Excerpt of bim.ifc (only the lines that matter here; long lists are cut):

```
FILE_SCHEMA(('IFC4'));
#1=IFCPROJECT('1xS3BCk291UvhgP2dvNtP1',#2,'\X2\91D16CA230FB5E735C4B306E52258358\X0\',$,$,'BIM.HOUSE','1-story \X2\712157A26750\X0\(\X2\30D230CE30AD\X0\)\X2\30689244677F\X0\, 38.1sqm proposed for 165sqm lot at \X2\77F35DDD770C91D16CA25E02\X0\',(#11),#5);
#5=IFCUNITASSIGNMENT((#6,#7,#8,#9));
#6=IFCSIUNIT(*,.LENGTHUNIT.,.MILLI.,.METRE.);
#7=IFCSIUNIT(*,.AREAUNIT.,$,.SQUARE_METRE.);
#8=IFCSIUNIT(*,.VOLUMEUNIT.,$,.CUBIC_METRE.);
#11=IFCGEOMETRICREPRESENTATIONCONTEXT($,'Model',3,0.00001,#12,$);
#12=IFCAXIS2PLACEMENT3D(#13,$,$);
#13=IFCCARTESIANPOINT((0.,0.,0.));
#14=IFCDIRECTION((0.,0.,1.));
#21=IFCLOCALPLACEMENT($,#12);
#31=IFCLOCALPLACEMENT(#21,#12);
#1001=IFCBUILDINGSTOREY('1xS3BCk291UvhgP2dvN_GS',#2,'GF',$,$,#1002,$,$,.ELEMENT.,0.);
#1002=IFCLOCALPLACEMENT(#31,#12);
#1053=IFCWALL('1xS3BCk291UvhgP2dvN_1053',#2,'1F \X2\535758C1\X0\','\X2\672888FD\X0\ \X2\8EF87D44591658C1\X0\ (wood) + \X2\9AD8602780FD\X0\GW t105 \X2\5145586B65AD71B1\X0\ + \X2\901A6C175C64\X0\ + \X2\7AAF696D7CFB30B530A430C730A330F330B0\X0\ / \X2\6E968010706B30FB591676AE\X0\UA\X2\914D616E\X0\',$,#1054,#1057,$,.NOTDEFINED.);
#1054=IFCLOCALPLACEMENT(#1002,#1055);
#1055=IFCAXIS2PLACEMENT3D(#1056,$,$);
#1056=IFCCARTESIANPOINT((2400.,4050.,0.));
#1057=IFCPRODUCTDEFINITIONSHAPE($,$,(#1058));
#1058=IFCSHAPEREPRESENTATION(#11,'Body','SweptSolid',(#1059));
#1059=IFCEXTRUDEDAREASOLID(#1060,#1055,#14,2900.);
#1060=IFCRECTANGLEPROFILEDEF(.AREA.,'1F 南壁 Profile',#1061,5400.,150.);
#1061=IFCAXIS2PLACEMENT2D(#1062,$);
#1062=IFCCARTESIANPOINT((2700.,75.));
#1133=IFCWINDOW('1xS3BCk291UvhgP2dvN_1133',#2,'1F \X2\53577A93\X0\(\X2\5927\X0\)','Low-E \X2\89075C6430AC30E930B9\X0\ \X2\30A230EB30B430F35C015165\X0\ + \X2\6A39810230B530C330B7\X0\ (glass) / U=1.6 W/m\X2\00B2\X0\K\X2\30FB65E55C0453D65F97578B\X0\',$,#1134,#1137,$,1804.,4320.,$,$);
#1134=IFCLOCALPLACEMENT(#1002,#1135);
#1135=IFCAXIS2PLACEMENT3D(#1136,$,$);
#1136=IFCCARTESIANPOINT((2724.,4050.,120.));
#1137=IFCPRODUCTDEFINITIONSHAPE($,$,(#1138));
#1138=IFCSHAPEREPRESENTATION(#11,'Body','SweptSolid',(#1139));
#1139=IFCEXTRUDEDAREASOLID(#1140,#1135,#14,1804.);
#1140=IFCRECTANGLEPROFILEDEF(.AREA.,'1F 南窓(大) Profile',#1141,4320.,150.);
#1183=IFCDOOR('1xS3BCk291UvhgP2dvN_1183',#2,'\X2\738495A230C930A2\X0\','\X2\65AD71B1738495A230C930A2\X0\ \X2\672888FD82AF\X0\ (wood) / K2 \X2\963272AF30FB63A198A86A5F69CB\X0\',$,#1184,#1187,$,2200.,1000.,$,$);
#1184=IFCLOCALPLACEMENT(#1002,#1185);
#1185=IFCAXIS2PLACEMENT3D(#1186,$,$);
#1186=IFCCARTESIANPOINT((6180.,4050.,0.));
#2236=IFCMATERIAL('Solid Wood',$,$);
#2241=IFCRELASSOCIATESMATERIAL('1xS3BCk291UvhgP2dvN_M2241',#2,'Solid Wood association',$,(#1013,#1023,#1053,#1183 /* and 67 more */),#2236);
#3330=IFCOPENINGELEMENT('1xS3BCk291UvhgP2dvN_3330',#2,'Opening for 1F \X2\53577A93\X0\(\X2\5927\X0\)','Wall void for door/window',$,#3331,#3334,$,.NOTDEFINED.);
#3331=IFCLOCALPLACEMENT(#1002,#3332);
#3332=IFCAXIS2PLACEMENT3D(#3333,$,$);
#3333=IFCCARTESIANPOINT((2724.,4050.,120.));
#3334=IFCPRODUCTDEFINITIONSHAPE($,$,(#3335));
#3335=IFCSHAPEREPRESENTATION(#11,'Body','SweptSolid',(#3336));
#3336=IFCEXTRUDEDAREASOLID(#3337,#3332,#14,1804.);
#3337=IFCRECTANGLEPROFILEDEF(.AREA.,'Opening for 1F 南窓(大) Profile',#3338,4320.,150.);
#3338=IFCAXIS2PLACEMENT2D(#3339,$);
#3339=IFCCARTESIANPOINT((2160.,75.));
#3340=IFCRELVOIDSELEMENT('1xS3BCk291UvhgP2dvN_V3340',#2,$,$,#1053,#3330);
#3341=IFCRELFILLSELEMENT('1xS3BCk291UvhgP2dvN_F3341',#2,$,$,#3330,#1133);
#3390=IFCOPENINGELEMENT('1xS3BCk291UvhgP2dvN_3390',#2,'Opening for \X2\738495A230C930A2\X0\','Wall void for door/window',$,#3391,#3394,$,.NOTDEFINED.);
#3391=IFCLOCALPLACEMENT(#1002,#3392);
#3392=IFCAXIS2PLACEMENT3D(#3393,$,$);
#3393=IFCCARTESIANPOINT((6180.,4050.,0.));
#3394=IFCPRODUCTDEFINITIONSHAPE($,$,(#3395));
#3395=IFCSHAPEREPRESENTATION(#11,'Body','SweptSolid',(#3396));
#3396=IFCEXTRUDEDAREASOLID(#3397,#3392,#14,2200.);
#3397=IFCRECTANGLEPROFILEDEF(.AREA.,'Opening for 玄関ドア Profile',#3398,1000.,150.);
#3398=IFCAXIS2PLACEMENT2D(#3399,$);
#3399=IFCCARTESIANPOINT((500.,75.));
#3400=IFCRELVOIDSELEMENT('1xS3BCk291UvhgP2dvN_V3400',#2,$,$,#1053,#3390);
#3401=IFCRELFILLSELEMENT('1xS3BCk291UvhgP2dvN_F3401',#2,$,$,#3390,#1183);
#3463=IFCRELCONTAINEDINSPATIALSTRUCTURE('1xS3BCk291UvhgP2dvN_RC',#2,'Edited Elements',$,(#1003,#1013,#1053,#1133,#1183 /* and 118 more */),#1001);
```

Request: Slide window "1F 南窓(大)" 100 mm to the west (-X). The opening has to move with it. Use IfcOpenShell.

```python
import ifcopenshell
import ifcopenshell.api.geometry
import ifcopenshell.util.placement

model = ifcopenshell.open("bim.ifc")

window = model.by_id(1133)
opening = window.FillsVoids[0].RelatingOpeningElement
wall = opening.VoidsElements[0].RelatingBuildingElement

wall_matrix = ifcopenshell.util.placement.get_local_placement(wall.ObjectPlacement)
shift = wall_matrix[:3, 0] * -100.0
before = ifcopenshell.util.placement.get_local_placement(window.ObjectPlacement)[:3, 3].copy()

# The window is not placed relative to its opening, so move both.
for product in (opening, window):
    matrix = ifcopenshell.util.placement.get_local_placement(product.ObjectPlacement)
    matrix[:3, 3] += shift
    ifcopenshell.api.geometry.edit_object_placement(model, product=product, matrix=matrix, is_si=False)

after = ifcopenshell.util.placement.get_local_placement(window.ObjectPlacement)[:3, 3]
print("window moved by", (after - before).round(3) + 0.0)

model.write("bim_rev.ifc")
```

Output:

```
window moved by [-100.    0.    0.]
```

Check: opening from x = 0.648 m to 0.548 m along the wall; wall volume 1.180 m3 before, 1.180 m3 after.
